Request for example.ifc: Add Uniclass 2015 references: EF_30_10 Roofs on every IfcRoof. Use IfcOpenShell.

First a look at what the model holds.

```python
import ifcopenshell

model = ifcopenshell.open("example.ifc")
print(model.schema)
print("classifications:", [c.Name for c in model.by_type("IfcClassification")])
for ifc_class in ("IfcDoor", "IfcRoof", "IfcStair", "IfcWall", "IfcWindow"):
    print(ifc_class, len(model.by_type(ifc_class)))
```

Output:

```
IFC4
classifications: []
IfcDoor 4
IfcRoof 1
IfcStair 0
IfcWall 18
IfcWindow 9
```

```python
import ifcopenshell
import ifcopenshell.api.classification

model = ifcopenshell.open("example.ifc")

system = ifcopenshell.api.classification.add_classification(model, classification="Uniclass 2015")

codes = {
    "IfcRoof": ("EF_30_10", "Roofs"),
}
for ifc_class, (code, name) in codes.items():
    products = model.by_type(ifc_class)
    ifcopenshell.api.classification.add_reference(
        model, products=products, classification=system, identification=code, name=name
    )
    print(code, len(products))

model.write("example_updated.ifc")
```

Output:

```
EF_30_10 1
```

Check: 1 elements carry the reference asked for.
